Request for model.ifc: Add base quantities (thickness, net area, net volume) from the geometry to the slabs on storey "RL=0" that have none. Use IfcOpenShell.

First a look at what the model holds.

```python
import ifcopenshell
import ifcopenshell.util.element
import ifcopenshell.util.unit

model = ifcopenshell.open("model.ifc")
print(model.schema)
for unit_type in ("LENGTHUNIT", "AREAUNIT", "VOLUMEUNIT"):
    print(unit_type, ifcopenshell.util.unit.calculate_unit_scale(model, unit_type))
storey = next(s for s in model.by_type("IfcBuildingStorey") if s.Name == "RL=0")
slabs = [e for e in ifcopenshell.util.element.get_decomposition(storey) if e.is_a("IfcSlab")]
for e in sorted(slabs, key=lambda e: e.id()):
    print(e.id(), e.is_a(), e.Name, list(ifcopenshell.util.element.get_psets(e, qtos_only=True)), sep=" | ")
```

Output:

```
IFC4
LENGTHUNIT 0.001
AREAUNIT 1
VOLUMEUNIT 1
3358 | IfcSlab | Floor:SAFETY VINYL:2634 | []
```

```python
import ifcopenshell
import ifcopenshell.api.pset
import ifcopenshell.geom
import ifcopenshell.util.element
import ifcopenshell.util.shape
import ifcopenshell.util.unit

model = ifcopenshell.open("model.ifc")
unit_scale = ifcopenshell.util.unit.calculate_unit_scale(model)
area_scale = ifcopenshell.util.unit.calculate_unit_scale(model, "AREAUNIT")
volume_scale = ifcopenshell.util.unit.calculate_unit_scale(model, "VOLUMEUNIT")
settings = ifcopenshell.geom.settings()

storey = next(s for s in model.by_type("IfcBuildingStorey") if s.Name == "RL=0")
slabs = [e for e in ifcopenshell.util.element.get_decomposition(storey) if e.is_a("IfcSlab")]

for e in sorted(slabs, key=lambda e: e.id()):
    if ifcopenshell.util.element.get_psets(e, qtos_only=True, should_inherit=False):
        continue
    # Geometry comes back in metres, in the element's own axes.
    shape = ifcopenshell.geom.create_shape(settings, e)
    values = {
        "Width": ifcopenshell.util.shape.get_z(shape.geometry) / unit_scale,
        "NetArea": ifcopenshell.util.shape.get_footprint_area(shape.geometry) / area_scale,
        "NetVolume": ifcopenshell.util.shape.get_volume(shape.geometry) / volume_scale,
    }
    qto = ifcopenshell.api.pset.add_qto(model, product=e, name="Qto_SlabBaseQuantities")
    ifcopenshell.api.pset.edit_qto(model, qto=qto, properties=values)
    print(e.id(), {k: round(v, 3) for k, v in values.items()})

model.write("model-out.ifc")
```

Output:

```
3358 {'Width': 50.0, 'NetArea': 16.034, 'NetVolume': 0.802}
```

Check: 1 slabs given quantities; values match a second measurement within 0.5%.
